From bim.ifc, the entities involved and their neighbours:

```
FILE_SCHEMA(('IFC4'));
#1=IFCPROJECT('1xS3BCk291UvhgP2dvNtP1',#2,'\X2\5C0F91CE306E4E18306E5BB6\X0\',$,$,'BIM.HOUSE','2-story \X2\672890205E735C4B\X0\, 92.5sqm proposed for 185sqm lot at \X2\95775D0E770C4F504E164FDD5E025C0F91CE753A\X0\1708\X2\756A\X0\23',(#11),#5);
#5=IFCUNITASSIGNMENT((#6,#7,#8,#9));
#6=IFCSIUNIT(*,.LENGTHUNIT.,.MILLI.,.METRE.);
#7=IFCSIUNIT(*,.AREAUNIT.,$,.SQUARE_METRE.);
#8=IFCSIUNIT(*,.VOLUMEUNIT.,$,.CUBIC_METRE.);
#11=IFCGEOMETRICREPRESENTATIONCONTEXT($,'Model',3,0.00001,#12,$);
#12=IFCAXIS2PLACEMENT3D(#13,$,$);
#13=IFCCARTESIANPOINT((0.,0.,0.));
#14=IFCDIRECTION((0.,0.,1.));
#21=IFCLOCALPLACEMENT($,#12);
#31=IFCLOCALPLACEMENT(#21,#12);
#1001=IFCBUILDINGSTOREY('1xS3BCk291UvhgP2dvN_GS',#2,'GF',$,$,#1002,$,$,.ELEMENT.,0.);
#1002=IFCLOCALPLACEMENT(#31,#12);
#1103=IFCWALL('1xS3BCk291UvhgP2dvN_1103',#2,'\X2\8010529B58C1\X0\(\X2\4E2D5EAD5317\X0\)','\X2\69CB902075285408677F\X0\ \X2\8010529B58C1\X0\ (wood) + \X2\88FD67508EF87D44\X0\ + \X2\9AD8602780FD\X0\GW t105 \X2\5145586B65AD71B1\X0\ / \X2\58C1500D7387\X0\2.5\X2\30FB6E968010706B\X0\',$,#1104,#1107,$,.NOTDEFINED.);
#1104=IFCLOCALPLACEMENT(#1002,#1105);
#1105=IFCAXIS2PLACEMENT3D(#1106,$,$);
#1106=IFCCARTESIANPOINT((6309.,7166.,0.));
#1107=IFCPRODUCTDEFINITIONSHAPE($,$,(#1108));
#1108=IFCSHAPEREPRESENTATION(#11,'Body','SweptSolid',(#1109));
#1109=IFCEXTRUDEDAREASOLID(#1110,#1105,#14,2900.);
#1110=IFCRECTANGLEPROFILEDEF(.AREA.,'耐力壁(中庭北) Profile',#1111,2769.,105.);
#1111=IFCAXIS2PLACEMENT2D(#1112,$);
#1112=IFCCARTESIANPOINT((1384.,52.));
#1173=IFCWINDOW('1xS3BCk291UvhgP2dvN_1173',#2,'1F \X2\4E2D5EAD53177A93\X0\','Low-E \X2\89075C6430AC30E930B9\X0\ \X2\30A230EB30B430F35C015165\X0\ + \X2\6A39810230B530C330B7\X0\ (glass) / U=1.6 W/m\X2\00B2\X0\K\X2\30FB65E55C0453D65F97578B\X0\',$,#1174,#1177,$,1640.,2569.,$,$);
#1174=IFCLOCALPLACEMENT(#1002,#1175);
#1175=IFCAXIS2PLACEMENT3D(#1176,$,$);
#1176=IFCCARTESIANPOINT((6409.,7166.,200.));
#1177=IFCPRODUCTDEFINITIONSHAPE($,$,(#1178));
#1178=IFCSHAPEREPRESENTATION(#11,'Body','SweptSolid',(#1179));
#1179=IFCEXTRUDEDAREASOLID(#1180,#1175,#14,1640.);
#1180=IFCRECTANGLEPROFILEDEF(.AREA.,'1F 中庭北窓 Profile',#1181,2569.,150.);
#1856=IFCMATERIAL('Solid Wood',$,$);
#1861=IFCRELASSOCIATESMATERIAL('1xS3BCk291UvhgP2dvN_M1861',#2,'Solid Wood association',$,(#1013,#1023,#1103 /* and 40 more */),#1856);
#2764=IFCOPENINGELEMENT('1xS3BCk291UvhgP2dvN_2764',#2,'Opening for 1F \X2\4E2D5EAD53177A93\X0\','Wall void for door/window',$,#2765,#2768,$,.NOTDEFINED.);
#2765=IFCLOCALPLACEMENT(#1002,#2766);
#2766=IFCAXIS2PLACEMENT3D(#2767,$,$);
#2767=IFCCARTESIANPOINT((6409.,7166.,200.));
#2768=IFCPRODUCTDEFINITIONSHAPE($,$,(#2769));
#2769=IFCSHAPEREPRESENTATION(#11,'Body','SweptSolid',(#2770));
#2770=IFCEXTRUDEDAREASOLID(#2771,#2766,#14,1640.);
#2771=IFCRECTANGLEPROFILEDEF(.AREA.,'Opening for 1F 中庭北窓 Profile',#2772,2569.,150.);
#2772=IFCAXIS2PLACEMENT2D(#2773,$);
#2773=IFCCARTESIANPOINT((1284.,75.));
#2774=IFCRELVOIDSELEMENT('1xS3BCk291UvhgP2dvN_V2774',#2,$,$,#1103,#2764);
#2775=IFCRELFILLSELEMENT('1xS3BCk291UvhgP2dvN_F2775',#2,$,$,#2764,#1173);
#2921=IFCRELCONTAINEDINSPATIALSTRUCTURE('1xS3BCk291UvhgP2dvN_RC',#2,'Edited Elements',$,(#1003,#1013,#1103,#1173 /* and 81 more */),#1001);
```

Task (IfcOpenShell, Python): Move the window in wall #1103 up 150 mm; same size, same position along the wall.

```python
import numpy as np
import ifcopenshell
import ifcopenshell.api.geometry
import ifcopenshell.util.placement
import ifcopenshell.util.unit

model = ifcopenshell.open("bim.ifc")
unit_scale = ifcopenshell.util.unit.calculate_unit_scale(model)

window = model.by_guid("1xS3BCk291UvhgP2dvN_1173")
opening = window.FillsVoids[0].RelatingOpeningElement
dz = 0.15 / unit_scale

shift = np.array([0.0, 0.0, dz])
# The window is not placed relative to its opening, so move both.
for product in (opening, window):
    matrix = ifcopenshell.util.placement.get_local_placement(product.ObjectPlacement)
    matrix[:3, 3] += shift
    ifcopenshell.api.geometry.edit_object_placement(model, product=product, matrix=matrix, is_si=False)

print(f"moved by {dz * unit_scale:+.3f} m")

model.write("bim-out.ifc")
```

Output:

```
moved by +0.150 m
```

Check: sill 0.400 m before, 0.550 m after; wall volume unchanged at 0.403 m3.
